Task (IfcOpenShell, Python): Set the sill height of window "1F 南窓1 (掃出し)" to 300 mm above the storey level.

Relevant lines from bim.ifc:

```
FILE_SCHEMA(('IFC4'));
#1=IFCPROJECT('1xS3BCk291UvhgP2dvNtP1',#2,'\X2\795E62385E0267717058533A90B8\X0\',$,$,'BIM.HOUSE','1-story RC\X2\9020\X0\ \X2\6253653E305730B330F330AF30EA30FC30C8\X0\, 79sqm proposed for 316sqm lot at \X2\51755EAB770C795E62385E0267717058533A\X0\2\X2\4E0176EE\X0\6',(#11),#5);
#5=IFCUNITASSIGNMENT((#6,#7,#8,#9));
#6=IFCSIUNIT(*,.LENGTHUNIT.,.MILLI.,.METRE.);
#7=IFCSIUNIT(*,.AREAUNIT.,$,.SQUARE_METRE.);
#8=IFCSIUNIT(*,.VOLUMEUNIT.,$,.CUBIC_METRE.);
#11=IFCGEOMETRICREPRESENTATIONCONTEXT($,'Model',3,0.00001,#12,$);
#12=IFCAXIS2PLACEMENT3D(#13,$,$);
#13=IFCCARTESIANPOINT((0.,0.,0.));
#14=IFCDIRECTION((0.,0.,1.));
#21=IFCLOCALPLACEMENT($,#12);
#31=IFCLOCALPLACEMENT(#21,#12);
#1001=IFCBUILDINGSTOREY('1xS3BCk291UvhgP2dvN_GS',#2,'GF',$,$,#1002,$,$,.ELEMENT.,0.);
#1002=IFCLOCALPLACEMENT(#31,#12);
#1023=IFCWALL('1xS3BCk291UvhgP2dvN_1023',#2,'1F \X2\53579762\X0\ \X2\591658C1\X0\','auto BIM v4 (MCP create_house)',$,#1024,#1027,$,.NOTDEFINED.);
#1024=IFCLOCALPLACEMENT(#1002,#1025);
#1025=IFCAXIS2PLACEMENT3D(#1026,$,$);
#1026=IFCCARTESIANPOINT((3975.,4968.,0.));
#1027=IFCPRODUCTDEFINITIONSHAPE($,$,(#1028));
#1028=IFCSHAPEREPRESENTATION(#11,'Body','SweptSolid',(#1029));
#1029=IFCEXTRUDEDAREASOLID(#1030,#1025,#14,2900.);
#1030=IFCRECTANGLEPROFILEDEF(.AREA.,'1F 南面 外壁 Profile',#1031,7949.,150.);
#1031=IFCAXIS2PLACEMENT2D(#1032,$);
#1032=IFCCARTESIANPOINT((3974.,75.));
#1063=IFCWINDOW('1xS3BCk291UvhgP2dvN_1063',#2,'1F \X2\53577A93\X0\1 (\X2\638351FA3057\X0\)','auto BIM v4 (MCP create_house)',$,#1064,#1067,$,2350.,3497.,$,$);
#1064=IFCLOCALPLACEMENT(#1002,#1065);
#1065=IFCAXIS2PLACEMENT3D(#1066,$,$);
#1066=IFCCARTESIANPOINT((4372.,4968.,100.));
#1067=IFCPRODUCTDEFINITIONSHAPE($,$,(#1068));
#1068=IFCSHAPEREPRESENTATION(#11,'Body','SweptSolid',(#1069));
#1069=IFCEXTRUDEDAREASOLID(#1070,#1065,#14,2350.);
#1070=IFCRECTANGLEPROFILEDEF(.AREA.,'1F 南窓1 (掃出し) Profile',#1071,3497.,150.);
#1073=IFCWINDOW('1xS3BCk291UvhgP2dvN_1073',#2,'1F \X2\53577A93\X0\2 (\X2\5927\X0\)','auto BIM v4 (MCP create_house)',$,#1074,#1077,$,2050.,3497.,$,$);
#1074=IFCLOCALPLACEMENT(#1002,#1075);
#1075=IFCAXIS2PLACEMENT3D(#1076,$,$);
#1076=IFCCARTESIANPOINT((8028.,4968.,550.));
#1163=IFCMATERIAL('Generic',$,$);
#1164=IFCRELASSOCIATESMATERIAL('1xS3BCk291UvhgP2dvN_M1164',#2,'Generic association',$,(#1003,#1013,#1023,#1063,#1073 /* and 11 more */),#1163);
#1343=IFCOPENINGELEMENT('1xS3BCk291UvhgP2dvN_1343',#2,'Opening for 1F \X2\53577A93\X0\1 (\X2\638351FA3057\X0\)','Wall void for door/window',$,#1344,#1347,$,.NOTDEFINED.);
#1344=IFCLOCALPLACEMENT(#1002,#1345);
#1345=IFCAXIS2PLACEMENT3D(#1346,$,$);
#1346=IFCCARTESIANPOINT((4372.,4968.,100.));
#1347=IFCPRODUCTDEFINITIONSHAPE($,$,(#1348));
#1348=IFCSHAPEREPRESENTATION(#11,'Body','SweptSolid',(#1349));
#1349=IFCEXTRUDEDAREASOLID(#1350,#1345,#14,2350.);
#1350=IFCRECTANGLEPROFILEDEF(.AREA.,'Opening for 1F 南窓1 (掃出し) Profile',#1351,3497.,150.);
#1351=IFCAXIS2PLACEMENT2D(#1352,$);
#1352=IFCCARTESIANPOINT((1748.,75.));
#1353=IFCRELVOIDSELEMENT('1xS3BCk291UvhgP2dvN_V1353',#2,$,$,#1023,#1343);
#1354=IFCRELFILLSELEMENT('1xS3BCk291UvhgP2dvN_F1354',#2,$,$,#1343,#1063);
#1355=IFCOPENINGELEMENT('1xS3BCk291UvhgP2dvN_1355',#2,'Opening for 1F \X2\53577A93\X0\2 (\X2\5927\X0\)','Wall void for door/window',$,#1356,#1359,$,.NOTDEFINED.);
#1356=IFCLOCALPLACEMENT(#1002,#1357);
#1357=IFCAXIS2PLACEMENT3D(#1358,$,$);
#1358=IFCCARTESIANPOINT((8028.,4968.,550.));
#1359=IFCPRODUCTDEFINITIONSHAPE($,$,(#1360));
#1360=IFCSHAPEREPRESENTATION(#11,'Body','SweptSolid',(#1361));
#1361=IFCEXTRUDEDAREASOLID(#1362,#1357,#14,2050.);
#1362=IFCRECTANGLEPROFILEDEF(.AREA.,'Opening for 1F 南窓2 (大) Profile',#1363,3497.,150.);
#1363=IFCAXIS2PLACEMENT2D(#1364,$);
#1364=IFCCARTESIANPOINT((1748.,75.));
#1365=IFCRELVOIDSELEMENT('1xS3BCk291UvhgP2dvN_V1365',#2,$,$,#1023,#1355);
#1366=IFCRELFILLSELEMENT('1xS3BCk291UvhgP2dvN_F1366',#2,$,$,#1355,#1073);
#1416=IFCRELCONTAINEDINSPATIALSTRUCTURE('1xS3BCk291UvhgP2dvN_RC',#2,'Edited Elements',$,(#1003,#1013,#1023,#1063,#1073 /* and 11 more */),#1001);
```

```python
import numpy as np
import ifcopenshell
import ifcopenshell.api.geometry
import ifcopenshell.geom
import ifcopenshell.util.element
import ifcopenshell.util.placement
import ifcopenshell.util.shape
import ifcopenshell.util.unit

model = ifcopenshell.open("bim.ifc")
unit_scale = ifcopenshell.util.unit.calculate_unit_scale(model)

window = model.by_guid("1xS3BCk291UvhgP2dvN_1063")
opening = window.FillsVoids[0].RelatingOpeningElement
storey = ifcopenshell.util.element.get_container(window, ifc_class="IfcBuildingStorey")
level = ifcopenshell.util.placement.get_local_placement(storey.ObjectPlacement)[2, 3]

# The opening's origin need not be at the sill, so measure its lowest point.
shape = ifcopenshell.geom.create_shape(ifcopenshell.geom.settings(), opening)
bottom = ifcopenshell.util.shape.get_shape_bottom_elevation(shape, shape.geometry) / unit_scale
dz = level + 0.3 / unit_scale - bottom

shift = np.array([0.0, 0.0, dz])
# The window is not placed relative to its opening, so move both.
for product in (opening, window):
    matrix = ifcopenshell.util.placement.get_local_placement(product.ObjectPlacement)
    matrix[:3, 3] += shift
    ifcopenshell.api.geometry.edit_object_placement(model, product=product, matrix=matrix, is_si=False)

print(f"moved by {dz * unit_scale:+.3f} m")

model.write("bim_rev.ifc")
```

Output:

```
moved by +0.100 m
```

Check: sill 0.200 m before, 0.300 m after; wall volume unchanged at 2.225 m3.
